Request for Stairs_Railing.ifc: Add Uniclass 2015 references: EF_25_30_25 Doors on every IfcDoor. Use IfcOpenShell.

First a look at what the model holds.

```python
import ifcopenshell

model = ifcopenshell.open("Stairs_Railing.ifc")
print(model.schema)
print("classifications:", [c.Name for c in model.by_type("IfcClassification")])
for ifc_class in ("IfcDoor", "IfcRoof", "IfcStair", "IfcWall", "IfcWindow"):
    print(ifc_class, len(model.by_type(ifc_class)))
```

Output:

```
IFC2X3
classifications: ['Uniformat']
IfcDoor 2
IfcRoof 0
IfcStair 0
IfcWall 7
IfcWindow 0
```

```python
import ifcopenshell
import ifcopenshell.api.classification

model = ifcopenshell.open("Stairs_Railing.ifc")

# IFC2X3 requires Source and Edition and has no link from the project to the system.
system = model.create_entity("IfcClassification", Source="NBS", Edition="2015", Name="Uniclass 2015")

codes = {
    "IfcDoor": ("EF_25_30_25", "Doors"),
}
for ifc_class, (code, name) in codes.items():
    products = model.by_type(ifc_class)
    ifcopenshell.api.classification.add_reference(
        model, products=products, classification=system, identification=code, name=name
    )
    print(code, len(products))

model.write("Stairs_Railing_rev.ifc")
```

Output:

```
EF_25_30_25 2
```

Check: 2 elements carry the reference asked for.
